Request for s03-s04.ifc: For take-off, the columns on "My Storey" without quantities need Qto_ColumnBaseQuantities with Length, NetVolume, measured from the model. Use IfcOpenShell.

First a look at what the model holds.

```python
import ifcopenshell
import ifcopenshell.util.element
import ifcopenshell.util.unit

model = ifcopenshell.open("s03-s04.ifc")
print(model.schema)
for unit_type in ("LENGTHUNIT", "AREAUNIT", "VOLUMEUNIT"):
    print(unit_type, ifcopenshell.util.unit.calculate_unit_scale(model, unit_type))
storey = next(s for s in model.by_type("IfcBuildingStorey") if s.Name == "My Storey")
columns = [e for e in ifcopenshell.util.element.get_decomposition(storey) if e.is_a("IfcColumn")]
for e in sorted(columns, key=lambda e: e.id()):
    print(e.id(), e.is_a(), e.Name, list(ifcopenshell.util.element.get_psets(e, qtos_only=True)), sep=" | ")
```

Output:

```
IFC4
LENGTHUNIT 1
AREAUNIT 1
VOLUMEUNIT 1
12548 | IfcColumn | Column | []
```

```python
import ifcopenshell
import ifcopenshell.api.pset
import ifcopenshell.geom
import ifcopenshell.util.element
import ifcopenshell.util.shape
import ifcopenshell.util.unit

model = ifcopenshell.open("s03-s04.ifc")
unit_scale = ifcopenshell.util.unit.calculate_unit_scale(model)
volume_scale = ifcopenshell.util.unit.calculate_unit_scale(model, "VOLUMEUNIT")
settings = ifcopenshell.geom.settings()

storey = next(s for s in model.by_type("IfcBuildingStorey") if s.Name == "My Storey")
columns = [e for e in ifcopenshell.util.element.get_decomposition(storey) if e.is_a("IfcColumn")]

for e in sorted(columns, key=lambda e: e.id()):
    if ifcopenshell.util.element.get_psets(e, qtos_only=True, should_inherit=False):
        continue
    # Geometry comes back in metres, in the element's own axes.
    shape = ifcopenshell.geom.create_shape(settings, e)
    values = {
        "Length": ifcopenshell.util.shape.get_z(shape.geometry) / unit_scale,
        "NetVolume": ifcopenshell.util.shape.get_volume(shape.geometry) / volume_scale,
    }
    qto = ifcopenshell.api.pset.add_qto(model, product=e, name="Qto_ColumnBaseQuantities")
    ifcopenshell.api.pset.edit_qto(model, qto=qto, properties=values)
    print(e.id(), {k: round(v, 3) for k, v in values.items()})

model.write("s03-s04_rev.ifc")
```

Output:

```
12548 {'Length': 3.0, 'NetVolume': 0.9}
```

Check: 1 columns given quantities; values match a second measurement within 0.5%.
